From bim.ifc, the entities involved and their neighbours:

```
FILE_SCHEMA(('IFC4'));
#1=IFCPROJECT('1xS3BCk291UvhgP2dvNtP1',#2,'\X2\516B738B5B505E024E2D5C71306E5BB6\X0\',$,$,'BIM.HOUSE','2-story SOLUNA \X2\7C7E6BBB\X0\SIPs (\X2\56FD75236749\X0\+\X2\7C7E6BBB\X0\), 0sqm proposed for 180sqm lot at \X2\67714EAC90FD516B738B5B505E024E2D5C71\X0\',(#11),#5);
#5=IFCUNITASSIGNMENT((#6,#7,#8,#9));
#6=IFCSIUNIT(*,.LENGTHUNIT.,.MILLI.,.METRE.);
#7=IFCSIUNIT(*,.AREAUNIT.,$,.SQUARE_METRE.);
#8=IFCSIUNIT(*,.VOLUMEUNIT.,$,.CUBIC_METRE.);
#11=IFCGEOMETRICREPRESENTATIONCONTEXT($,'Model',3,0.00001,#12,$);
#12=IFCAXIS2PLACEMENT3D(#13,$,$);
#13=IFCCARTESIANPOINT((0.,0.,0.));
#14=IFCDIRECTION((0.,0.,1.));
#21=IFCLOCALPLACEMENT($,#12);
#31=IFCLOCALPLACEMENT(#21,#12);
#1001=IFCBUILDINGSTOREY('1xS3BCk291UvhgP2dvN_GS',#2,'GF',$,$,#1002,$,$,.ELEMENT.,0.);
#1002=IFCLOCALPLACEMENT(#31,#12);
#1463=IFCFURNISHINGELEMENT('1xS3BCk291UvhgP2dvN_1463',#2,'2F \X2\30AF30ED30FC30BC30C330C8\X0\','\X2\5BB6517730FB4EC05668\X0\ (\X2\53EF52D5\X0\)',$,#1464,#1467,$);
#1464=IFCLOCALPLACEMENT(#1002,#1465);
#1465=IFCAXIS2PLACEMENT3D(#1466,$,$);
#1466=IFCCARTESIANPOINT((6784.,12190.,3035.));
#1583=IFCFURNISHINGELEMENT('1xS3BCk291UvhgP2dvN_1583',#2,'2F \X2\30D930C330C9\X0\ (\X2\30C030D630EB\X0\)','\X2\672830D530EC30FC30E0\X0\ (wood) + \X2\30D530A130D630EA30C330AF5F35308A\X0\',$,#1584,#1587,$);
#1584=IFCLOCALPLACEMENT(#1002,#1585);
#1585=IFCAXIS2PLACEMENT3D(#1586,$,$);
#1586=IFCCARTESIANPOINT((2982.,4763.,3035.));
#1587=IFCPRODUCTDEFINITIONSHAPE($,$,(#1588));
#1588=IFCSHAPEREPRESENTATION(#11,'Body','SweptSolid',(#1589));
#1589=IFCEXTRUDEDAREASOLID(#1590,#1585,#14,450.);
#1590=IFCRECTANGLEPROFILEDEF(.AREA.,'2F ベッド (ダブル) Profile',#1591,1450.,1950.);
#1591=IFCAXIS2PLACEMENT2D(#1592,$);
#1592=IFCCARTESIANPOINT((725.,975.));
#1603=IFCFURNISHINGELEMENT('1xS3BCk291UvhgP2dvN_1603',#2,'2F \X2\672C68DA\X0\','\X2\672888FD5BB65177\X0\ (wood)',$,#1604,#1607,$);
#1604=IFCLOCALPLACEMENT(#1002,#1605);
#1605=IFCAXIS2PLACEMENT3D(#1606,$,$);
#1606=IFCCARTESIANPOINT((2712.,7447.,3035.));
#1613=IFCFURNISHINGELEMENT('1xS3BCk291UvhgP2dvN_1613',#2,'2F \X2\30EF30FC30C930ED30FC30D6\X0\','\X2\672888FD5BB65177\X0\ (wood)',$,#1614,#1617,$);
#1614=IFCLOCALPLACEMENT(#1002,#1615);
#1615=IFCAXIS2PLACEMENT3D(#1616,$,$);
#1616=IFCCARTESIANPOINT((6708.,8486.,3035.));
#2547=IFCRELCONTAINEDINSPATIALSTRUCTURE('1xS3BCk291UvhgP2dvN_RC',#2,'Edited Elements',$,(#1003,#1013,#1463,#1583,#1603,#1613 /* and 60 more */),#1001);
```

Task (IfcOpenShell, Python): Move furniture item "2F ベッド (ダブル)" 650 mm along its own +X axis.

```python
import ifcopenshell
import ifcopenshell.api.geometry
import ifcopenshell.util.placement

model = ifcopenshell.open("bim.ifc")

item = model.by_id(1583)
matrix = ifcopenshell.util.placement.get_local_placement(item.ObjectPlacement)
matrix[:3, 3] += matrix[:3, 0] * 650.0
ifcopenshell.api.geometry.edit_object_placement(model, product=item, matrix=matrix, is_si=False)

print(ifcopenshell.util.placement.get_local_placement(item.ObjectPlacement).round(3) + 0.0)

model.write("bim_edited.ifc")
```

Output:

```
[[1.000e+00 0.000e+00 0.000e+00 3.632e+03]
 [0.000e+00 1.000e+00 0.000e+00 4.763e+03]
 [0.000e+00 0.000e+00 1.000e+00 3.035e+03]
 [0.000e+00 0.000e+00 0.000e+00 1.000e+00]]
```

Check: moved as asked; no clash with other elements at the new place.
